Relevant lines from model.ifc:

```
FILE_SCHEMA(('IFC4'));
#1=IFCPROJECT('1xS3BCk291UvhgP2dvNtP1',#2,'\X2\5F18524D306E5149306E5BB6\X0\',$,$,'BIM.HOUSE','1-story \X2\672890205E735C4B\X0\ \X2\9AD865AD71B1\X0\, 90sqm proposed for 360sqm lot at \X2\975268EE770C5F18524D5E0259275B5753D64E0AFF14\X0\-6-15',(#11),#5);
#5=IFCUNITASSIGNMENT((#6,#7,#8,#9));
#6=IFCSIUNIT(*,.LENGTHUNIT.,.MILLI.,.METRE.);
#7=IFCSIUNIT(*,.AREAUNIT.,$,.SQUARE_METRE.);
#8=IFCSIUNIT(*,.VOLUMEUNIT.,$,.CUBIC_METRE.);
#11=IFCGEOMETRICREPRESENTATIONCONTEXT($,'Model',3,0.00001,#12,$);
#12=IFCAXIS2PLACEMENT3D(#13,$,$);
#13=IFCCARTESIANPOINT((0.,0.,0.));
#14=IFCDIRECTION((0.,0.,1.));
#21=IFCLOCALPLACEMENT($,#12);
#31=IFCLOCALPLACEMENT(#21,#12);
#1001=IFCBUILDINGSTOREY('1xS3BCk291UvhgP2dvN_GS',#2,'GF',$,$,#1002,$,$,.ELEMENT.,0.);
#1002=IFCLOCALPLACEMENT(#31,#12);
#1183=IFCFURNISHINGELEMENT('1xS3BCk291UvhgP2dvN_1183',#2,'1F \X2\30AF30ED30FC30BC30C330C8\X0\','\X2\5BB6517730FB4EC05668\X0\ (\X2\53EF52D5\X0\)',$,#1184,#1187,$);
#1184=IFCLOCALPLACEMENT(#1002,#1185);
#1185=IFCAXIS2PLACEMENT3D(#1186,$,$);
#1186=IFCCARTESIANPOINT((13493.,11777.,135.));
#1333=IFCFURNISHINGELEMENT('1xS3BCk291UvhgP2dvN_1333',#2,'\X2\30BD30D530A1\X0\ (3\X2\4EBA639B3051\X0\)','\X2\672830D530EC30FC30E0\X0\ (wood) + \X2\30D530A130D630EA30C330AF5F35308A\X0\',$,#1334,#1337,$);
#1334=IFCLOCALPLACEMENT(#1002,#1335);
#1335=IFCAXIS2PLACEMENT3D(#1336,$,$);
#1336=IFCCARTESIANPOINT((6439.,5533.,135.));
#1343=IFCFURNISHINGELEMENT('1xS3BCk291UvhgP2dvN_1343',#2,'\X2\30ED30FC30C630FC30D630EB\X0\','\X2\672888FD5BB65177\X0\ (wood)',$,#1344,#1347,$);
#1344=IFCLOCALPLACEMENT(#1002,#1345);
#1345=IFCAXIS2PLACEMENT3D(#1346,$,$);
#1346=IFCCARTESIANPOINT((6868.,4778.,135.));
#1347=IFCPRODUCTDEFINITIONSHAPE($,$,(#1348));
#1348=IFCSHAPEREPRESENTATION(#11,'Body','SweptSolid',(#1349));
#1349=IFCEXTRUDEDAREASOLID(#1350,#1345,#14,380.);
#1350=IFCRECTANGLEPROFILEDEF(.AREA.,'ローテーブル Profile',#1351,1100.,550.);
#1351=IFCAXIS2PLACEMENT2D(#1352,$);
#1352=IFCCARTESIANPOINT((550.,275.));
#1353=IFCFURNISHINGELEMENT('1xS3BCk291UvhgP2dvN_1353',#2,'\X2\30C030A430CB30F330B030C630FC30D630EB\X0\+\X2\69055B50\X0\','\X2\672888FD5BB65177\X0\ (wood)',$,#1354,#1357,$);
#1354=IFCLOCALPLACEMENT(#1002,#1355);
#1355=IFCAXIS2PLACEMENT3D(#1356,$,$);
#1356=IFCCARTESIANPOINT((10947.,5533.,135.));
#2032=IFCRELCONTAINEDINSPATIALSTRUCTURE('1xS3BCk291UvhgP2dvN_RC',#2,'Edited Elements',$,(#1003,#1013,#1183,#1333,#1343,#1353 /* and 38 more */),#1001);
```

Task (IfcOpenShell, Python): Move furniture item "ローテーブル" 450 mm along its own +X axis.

```python
import ifcopenshell
import ifcopenshell.api.geometry
import ifcopenshell.util.placement

model = ifcopenshell.open("model.ifc")

item = model.by_guid("1xS3BCk291UvhgP2dvN_1343")
matrix = ifcopenshell.util.placement.get_local_placement(item.ObjectPlacement)
matrix[:3, 3] += matrix[:3, 0] * 450.0
ifcopenshell.api.geometry.edit_object_placement(model, product=item, matrix=matrix, is_si=False)

print(ifcopenshell.util.placement.get_local_placement(item.ObjectPlacement).round(3) + 0.0)

model.write("model_rev.ifc")
```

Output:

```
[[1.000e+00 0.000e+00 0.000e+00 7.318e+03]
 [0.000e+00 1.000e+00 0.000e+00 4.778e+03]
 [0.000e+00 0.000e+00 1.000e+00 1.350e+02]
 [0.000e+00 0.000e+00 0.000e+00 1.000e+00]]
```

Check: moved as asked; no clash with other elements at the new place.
